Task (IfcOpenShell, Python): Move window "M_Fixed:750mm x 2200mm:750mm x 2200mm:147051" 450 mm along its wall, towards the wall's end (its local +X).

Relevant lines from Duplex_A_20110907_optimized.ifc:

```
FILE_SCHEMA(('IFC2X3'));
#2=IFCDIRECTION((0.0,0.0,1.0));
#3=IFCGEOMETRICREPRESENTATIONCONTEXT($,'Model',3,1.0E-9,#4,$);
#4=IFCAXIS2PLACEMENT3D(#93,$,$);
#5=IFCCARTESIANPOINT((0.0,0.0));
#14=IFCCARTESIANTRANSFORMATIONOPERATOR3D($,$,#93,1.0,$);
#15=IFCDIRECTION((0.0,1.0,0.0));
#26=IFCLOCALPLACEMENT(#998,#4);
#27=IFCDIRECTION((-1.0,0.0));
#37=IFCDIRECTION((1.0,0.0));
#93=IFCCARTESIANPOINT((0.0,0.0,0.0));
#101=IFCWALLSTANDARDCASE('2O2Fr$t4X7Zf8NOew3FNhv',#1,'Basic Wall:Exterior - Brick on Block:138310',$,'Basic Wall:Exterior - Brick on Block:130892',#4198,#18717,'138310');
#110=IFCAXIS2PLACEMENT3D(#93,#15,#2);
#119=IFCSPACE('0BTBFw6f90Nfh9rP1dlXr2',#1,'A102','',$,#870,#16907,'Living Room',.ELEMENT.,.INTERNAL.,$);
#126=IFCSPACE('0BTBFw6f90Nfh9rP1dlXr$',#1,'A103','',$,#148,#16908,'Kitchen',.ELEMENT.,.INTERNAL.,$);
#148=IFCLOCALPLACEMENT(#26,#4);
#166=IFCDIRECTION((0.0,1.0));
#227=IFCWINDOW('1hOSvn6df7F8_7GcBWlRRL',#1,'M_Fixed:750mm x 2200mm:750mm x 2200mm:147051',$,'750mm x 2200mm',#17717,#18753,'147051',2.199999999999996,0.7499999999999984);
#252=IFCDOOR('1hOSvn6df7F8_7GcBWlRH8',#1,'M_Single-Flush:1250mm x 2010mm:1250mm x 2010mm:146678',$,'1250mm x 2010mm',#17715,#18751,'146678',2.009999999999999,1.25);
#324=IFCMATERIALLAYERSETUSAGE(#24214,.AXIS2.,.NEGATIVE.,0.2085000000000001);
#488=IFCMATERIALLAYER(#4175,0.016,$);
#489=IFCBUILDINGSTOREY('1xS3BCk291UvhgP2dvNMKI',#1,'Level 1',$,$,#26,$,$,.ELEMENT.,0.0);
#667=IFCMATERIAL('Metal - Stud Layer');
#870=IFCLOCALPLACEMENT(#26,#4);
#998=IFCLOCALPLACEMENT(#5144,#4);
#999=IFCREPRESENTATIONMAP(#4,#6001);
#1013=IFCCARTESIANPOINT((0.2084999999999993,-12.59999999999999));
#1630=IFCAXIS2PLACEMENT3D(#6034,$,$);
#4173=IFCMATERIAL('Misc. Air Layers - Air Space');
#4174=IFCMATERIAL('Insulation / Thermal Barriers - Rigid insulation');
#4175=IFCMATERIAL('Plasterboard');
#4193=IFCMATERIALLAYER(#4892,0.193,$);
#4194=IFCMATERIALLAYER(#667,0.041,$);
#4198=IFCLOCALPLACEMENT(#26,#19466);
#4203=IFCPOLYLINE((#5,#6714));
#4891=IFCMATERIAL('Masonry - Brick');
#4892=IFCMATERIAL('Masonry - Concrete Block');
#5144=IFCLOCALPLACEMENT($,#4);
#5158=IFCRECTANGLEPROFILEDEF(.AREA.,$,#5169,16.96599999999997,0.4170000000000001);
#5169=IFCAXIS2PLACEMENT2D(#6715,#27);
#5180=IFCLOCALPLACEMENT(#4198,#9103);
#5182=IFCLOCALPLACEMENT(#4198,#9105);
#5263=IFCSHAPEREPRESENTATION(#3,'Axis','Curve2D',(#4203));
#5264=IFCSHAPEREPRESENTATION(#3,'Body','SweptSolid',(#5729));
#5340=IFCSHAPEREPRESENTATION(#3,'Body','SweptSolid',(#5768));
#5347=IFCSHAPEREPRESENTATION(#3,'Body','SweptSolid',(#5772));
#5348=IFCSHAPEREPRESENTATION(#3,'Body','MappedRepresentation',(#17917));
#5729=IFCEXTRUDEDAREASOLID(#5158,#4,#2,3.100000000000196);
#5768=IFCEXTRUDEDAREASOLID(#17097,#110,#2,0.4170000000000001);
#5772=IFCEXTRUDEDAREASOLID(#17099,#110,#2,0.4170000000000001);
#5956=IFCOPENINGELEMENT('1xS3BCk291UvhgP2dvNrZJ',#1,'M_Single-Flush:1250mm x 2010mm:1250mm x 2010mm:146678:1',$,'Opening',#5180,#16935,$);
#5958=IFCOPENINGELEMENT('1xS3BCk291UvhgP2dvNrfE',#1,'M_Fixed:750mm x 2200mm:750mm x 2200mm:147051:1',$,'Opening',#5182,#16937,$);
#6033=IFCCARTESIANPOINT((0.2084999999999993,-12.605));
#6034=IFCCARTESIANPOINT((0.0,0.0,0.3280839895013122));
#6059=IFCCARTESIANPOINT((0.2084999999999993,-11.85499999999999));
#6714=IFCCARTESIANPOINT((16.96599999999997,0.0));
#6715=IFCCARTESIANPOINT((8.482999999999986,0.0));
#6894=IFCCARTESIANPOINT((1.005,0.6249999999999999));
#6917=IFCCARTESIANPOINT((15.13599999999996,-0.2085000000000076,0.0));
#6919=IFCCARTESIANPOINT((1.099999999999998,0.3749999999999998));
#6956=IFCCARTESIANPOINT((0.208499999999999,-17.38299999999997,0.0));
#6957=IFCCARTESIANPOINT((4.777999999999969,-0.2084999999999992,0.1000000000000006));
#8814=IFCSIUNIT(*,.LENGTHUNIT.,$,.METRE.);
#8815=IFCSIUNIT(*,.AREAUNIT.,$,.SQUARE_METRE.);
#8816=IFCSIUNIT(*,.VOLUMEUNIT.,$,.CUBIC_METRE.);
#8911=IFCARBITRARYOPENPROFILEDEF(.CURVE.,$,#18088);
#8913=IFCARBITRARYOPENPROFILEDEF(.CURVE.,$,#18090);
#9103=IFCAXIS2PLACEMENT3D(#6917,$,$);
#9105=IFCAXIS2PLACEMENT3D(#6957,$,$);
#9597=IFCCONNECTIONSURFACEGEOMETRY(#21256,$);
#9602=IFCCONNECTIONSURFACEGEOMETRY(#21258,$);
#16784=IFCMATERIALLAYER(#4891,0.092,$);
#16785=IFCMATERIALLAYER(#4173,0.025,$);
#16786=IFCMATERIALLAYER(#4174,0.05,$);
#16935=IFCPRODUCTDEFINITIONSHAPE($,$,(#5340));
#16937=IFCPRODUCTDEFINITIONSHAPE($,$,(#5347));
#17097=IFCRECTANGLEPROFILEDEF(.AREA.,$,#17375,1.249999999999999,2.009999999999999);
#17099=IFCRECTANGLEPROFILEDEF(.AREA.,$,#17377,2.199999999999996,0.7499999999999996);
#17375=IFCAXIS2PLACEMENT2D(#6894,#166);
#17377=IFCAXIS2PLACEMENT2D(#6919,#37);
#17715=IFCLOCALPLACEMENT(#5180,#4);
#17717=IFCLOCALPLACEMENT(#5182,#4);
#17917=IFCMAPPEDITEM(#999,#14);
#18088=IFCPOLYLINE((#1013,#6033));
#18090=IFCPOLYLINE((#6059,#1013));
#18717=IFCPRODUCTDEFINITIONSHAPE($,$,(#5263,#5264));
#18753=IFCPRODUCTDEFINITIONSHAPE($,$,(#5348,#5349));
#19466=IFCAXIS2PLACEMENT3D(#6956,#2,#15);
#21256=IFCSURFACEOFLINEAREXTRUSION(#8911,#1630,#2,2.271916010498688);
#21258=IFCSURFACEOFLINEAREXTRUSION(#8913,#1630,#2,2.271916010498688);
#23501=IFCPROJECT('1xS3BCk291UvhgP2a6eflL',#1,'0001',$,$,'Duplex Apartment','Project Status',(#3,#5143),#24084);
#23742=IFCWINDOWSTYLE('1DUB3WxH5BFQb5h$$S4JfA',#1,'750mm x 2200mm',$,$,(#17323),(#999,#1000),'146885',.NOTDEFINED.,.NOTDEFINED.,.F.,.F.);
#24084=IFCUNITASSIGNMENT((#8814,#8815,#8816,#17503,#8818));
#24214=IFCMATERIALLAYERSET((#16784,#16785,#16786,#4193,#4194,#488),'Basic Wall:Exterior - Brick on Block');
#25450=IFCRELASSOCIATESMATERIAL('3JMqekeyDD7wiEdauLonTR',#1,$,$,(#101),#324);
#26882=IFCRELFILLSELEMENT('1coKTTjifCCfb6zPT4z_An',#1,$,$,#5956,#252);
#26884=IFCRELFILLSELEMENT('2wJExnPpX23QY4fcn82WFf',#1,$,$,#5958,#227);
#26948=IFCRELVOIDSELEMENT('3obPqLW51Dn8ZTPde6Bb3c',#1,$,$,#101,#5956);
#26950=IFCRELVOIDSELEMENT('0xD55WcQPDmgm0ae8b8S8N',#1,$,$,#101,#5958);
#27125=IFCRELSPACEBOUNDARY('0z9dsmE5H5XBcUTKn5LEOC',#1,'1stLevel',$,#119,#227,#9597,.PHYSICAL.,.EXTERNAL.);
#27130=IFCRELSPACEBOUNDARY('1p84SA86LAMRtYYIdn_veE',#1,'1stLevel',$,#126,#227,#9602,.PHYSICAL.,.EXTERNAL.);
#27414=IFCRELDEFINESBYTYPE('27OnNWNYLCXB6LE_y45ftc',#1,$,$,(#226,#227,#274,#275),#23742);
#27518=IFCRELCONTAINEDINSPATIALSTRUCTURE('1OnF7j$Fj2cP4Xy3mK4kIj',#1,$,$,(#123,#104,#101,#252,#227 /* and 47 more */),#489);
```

```python
import numpy as np
import ifcopenshell
import ifcopenshell.api.geometry
import ifcopenshell.util.placement
import ifcopenshell.util.unit

model = ifcopenshell.open("Duplex_A_20110907_optimized.ifc")
unit_scale = ifcopenshell.util.unit.calculate_unit_scale(model)

window = model.by_guid("1hOSvn6df7F8_7GcBWlRRL")
opening = window.FillsVoids[0].RelatingOpeningElement
wall = opening.VoidsElements[0].RelatingBuildingElement

wall_matrix = ifcopenshell.util.placement.get_local_placement(wall.ObjectPlacement)
shift = wall_matrix[:3, 0] * 0.45 / unit_scale
before = ifcopenshell.util.placement.get_local_placement(window.ObjectPlacement)[:3, 3].copy()

# The window is placed relative to its opening, so it follows when the opening moves.
matrix = ifcopenshell.util.placement.get_local_placement(opening.ObjectPlacement)
matrix[:3, 3] += shift
ifcopenshell.api.geometry.edit_object_placement(
    model, product=opening, matrix=matrix, is_si=False, should_transform_children=True
)

# Space boundary surfaces are stored in each space's coordinates; move them too.
for rel in window.ProvidesBoundaries:
    if not rel.ConnectionGeometry:
        continue
    surface = rel.ConnectionGeometry.SurfaceOnRelatingElement
    space_matrix = ifcopenshell.util.placement.get_local_placement(rel.RelatingSpace.ObjectPlacement)
    point = np.array(surface.Position.Location.Coordinates) + space_matrix[:3, :3].T @ shift
    surface.Position = model.createIfcAxis2Placement3D(
        model.createIfcCartesianPoint(point.tolist()), surface.Position.Axis, surface.Position.RefDirection
    )

after = ifcopenshell.util.placement.get_local_placement(window.ObjectPlacement)[:3, 3]
print("window moved by", (after - before).round(3) + 0.0)

model.write("Duplex_A_20110907_optimized_updated.ifc")
```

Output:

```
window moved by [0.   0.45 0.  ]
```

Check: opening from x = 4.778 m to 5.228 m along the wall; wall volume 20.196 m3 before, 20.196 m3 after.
